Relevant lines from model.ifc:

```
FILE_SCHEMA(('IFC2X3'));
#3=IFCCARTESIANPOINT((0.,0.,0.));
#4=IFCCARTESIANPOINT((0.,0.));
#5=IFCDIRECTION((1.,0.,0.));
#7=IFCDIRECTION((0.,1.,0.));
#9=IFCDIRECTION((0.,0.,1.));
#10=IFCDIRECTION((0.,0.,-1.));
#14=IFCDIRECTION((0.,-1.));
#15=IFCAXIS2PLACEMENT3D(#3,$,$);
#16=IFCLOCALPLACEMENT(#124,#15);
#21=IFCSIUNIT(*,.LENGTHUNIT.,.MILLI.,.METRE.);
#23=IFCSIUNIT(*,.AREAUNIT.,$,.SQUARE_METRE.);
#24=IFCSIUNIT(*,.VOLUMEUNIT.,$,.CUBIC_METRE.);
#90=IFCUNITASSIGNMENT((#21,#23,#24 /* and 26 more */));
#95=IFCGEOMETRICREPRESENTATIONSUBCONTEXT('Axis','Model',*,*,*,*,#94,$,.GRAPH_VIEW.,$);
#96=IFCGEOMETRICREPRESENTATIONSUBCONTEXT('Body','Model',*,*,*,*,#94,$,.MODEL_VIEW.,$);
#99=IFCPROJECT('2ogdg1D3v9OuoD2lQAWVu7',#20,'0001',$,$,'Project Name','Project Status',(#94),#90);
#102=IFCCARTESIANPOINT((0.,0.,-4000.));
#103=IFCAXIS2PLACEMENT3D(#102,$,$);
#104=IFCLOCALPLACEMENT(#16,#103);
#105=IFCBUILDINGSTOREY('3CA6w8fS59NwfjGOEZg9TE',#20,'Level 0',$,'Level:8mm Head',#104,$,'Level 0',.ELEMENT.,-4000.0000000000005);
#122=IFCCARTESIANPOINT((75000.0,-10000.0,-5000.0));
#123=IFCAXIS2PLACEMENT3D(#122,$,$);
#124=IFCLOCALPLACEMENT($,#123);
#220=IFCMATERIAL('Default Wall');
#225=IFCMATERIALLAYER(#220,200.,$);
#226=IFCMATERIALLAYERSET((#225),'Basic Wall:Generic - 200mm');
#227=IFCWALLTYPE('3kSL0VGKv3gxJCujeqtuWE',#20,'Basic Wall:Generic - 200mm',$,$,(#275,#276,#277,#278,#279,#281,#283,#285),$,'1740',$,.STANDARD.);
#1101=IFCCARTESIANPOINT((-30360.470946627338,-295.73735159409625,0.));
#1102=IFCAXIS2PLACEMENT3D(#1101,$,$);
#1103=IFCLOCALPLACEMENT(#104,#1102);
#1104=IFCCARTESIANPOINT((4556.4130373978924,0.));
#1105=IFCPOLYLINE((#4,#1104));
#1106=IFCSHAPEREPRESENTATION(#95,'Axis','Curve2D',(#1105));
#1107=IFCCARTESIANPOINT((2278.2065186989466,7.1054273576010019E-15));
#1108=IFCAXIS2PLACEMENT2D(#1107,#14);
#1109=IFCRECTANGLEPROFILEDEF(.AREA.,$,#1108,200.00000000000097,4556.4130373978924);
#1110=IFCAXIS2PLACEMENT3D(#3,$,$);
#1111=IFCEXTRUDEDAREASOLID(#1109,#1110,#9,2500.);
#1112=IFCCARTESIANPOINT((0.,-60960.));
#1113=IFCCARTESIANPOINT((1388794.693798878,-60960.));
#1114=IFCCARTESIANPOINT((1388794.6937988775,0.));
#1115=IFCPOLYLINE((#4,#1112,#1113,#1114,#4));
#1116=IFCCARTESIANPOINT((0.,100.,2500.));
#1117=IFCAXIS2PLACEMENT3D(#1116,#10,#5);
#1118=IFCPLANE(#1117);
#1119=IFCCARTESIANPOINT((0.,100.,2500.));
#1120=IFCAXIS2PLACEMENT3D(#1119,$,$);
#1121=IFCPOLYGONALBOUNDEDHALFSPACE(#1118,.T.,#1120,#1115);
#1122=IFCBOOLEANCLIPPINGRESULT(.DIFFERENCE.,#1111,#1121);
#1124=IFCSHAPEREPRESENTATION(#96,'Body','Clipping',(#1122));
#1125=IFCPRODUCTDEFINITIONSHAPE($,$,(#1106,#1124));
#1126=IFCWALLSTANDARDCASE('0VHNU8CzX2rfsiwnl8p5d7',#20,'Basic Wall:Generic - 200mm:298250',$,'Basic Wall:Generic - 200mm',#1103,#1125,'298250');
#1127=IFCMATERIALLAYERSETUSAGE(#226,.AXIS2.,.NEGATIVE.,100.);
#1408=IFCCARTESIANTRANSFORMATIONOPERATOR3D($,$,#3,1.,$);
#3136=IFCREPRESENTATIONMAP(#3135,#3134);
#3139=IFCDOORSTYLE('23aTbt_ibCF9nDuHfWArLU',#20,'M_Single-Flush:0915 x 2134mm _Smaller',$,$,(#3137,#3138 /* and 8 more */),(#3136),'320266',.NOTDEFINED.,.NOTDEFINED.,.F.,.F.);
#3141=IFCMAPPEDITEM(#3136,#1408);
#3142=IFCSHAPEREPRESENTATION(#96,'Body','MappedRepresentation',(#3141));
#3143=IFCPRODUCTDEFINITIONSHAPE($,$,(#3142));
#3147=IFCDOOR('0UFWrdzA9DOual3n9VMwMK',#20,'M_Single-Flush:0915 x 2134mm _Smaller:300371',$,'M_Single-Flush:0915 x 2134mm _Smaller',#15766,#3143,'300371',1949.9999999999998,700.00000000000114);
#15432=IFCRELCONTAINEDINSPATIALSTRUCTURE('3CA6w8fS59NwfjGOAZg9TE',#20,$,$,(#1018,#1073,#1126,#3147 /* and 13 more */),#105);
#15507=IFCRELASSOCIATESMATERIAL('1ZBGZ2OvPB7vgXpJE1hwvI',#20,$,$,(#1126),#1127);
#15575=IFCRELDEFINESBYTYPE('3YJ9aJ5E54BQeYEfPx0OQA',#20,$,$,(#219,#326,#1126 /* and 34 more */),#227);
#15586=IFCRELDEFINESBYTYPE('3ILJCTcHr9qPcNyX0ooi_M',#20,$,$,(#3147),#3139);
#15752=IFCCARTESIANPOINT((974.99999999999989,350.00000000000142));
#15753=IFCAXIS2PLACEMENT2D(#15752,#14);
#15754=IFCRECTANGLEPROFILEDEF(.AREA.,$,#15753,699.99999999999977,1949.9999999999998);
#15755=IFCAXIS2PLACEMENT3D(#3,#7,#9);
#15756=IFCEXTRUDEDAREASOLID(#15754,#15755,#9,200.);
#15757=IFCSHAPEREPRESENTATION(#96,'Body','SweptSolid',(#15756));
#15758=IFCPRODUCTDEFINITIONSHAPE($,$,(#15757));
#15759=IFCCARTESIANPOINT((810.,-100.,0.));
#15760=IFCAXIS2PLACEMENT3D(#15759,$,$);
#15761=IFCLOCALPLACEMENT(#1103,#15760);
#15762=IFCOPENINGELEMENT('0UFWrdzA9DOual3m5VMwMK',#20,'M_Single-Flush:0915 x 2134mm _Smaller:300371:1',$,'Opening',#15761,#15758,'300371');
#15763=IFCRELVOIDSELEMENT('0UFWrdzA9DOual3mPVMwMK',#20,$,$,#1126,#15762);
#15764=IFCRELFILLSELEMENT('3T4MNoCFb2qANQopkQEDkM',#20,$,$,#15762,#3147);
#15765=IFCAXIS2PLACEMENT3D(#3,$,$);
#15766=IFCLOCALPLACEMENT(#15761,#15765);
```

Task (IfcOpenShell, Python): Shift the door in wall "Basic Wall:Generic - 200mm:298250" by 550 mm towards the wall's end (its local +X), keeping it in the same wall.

```python
import ifcopenshell
import ifcopenshell.api.geometry
import ifcopenshell.util.placement
import ifcopenshell.util.unit

model = ifcopenshell.open("model.ifc")
unit_scale = ifcopenshell.util.unit.calculate_unit_scale(model)

door = model.by_guid("0UFWrdzA9DOual3n9VMwMK")
opening = door.FillsVoids[0].RelatingOpeningElement
wall = opening.VoidsElements[0].RelatingBuildingElement

wall_matrix = ifcopenshell.util.placement.get_local_placement(wall.ObjectPlacement)
shift = wall_matrix[:3, 0] * 0.55 / unit_scale
before = ifcopenshell.util.placement.get_local_placement(door.ObjectPlacement)[:3, 3].copy()

# The door is placed relative to its opening, so it follows when the opening moves.
matrix = ifcopenshell.util.placement.get_local_placement(opening.ObjectPlacement)
matrix[:3, 3] += shift
ifcopenshell.api.geometry.edit_object_placement(
    model, product=opening, matrix=matrix, is_si=False, should_transform_children=True
)

after = ifcopenshell.util.placement.get_local_placement(door.ObjectPlacement)[:3, 3]
print("door moved by", (after - before).round(3) + 0.0)

model.write("model_rev.ifc")
```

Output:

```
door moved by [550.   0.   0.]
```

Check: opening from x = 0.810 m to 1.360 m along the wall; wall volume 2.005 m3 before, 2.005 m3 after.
